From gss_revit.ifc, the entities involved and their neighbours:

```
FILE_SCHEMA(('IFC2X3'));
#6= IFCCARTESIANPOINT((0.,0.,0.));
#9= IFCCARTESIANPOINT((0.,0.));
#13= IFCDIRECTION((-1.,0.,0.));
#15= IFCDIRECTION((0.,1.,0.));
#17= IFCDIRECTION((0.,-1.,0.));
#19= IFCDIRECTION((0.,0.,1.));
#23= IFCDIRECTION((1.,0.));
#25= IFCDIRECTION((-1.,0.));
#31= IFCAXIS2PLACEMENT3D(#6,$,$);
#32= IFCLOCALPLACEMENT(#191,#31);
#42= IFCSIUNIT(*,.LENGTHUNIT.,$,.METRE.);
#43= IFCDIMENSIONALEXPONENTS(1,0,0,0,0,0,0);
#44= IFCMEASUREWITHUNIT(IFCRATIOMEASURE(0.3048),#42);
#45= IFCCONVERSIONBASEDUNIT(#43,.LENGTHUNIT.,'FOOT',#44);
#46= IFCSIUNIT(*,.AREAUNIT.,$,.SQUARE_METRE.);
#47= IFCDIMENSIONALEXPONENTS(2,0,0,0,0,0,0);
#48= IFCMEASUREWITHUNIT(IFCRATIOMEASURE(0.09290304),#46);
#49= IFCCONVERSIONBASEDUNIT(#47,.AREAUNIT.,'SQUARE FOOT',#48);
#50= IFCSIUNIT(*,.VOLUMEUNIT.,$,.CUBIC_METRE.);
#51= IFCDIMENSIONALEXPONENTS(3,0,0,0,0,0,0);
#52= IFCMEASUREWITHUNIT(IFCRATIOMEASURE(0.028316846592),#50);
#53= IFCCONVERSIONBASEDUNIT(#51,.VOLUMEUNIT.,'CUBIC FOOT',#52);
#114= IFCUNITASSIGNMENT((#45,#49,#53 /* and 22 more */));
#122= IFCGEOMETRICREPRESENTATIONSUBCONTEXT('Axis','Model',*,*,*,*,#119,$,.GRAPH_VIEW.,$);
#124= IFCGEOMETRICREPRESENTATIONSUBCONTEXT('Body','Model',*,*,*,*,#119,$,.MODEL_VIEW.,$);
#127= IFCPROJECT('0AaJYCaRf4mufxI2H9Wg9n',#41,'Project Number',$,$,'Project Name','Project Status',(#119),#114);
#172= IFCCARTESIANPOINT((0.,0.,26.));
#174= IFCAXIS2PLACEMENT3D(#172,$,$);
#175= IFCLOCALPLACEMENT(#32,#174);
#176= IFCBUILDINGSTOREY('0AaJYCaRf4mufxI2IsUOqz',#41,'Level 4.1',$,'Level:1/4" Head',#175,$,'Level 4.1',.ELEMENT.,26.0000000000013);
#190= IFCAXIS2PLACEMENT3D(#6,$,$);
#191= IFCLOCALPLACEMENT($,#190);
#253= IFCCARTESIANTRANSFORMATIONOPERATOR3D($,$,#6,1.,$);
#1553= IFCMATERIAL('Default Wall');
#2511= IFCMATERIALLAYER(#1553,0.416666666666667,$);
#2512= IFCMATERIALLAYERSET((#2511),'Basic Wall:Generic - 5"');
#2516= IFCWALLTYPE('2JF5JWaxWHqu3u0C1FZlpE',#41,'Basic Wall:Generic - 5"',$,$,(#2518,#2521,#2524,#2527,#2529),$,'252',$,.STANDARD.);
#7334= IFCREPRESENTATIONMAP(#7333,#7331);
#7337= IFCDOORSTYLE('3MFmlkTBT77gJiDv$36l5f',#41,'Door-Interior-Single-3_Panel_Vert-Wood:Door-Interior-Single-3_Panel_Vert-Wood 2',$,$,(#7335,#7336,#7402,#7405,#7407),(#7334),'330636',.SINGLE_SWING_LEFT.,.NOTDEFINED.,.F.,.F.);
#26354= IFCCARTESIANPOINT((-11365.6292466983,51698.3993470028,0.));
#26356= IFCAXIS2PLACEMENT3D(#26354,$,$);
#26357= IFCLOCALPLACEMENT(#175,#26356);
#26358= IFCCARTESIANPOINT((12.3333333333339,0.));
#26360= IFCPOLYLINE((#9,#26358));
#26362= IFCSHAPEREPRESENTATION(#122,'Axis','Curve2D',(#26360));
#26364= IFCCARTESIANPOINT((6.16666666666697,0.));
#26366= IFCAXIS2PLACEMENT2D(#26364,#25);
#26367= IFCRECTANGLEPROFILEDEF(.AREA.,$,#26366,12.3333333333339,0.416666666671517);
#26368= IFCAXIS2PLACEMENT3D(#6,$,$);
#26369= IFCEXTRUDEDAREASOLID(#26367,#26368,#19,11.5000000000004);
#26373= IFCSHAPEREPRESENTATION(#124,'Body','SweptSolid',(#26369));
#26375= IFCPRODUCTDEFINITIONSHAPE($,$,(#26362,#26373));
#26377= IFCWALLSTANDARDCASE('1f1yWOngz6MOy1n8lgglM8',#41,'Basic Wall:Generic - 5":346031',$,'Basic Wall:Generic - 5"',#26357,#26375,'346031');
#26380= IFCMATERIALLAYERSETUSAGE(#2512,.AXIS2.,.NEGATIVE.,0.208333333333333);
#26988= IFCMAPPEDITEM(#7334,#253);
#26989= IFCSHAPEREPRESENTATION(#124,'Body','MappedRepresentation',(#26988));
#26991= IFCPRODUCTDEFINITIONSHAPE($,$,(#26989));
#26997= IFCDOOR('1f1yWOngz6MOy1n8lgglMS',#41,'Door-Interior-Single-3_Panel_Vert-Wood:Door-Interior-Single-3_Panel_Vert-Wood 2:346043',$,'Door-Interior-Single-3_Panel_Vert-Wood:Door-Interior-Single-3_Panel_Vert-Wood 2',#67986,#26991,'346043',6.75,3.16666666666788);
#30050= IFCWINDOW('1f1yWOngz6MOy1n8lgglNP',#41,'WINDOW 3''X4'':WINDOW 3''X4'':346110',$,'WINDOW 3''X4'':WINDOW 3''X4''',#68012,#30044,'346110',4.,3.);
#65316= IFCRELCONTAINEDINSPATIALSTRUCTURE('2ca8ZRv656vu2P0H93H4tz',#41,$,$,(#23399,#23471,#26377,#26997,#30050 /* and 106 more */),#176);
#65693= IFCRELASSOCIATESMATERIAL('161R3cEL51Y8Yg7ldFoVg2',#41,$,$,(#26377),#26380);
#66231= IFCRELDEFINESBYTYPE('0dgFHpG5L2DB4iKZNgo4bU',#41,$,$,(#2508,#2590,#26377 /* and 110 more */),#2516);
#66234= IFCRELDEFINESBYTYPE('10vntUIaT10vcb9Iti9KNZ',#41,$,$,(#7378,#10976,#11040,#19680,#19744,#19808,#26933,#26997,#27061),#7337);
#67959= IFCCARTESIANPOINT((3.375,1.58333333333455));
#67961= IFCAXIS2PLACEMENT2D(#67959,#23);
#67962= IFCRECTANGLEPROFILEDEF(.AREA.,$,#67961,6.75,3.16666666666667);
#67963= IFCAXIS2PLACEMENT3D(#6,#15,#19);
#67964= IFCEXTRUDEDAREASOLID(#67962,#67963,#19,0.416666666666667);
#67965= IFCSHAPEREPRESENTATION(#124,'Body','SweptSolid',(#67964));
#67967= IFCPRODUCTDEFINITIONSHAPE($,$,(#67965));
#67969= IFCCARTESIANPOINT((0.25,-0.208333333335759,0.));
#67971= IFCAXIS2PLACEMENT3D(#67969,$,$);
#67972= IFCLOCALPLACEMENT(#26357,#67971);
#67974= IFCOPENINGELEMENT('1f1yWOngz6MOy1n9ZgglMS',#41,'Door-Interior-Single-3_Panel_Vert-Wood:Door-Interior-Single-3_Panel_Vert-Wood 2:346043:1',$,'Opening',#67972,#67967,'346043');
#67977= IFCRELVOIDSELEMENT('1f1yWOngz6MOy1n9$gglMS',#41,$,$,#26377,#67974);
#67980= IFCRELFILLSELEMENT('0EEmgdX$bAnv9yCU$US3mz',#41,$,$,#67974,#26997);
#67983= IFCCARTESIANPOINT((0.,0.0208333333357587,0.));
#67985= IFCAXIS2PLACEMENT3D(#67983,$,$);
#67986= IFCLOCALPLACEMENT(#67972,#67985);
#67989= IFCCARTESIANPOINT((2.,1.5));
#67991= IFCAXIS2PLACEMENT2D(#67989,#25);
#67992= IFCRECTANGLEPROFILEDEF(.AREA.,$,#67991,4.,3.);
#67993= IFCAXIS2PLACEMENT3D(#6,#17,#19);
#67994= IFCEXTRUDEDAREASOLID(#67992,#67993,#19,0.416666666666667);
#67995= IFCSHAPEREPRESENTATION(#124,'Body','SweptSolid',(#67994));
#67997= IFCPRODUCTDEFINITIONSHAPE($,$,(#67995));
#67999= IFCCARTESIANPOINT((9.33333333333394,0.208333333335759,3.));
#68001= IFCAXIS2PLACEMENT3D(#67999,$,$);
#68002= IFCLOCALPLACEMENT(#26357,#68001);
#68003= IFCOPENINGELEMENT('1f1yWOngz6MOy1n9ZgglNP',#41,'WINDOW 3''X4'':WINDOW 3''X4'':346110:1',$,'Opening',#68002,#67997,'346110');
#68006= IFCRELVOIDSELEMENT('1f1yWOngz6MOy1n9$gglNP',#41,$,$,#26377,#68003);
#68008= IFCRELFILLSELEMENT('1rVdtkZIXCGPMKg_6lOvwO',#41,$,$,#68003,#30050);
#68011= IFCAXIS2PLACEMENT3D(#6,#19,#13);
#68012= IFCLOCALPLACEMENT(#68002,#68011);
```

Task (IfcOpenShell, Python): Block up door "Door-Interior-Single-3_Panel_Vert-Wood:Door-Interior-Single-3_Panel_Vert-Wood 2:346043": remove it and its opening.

```python
import ifcopenshell
import ifcopenshell.api.feature
import ifcopenshell.api.root
import ifcopenshell.geom
import ifcopenshell.util.shape

model = ifcopenshell.open("gss_revit.ifc")
settings = ifcopenshell.geom.settings()


def volume(element):
    """Net volume in cubic metres, openings subtracted."""
    shape = ifcopenshell.geom.create_shape(settings, element)
    return ifcopenshell.util.shape.get_volume(shape.geometry)


door = model.by_guid("1f1yWOngz6MOy1n8lgglMS")
opening = door.FillsVoids[0].RelatingOpeningElement
wall = opening.VoidsElements[0].RelatingBuildingElement
before = volume(wall)

ifcopenshell.api.root.remove_product(model, product=door)
ifcopenshell.api.feature.remove_feature(model, feature=opening)

after = volume(wall)

print(f"wall volume {before:.3f} -> {after:.3f} m3")

model.write("gss_revit-out.ifc")
```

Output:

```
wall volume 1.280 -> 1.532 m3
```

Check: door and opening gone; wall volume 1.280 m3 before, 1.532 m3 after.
